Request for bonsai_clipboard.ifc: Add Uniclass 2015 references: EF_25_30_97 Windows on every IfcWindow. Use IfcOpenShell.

First a look at what the model holds.

```python
import ifcopenshell

model = ifcopenshell.open("bonsai_clipboard.ifc")
print(model.schema)
print("classifications:", [c.Name for c in model.by_type("IfcClassification")])
for ifc_class in ("IfcDoor", "IfcRoof", "IfcStair", "IfcWall", "IfcWindow"):
    print(ifc_class, len(model.by_type(ifc_class)))
```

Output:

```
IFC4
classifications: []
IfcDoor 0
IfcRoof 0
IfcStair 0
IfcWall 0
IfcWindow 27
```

```python
import ifcopenshell
import ifcopenshell.api.classification

model = ifcopenshell.open("bonsai_clipboard.ifc")

system = ifcopenshell.api.classification.add_classification(model, classification="Uniclass 2015")

codes = {
    "IfcWindow": ("EF_25_30_97", "Windows"),
}
for ifc_class, (code, name) in codes.items():
    products = model.by_type(ifc_class)
    ifcopenshell.api.classification.add_reference(
        model, products=products, classification=system, identification=code, name=name
    )
    print(code, len(products))

model.write("bonsai_clipboard_v2.ifc")
```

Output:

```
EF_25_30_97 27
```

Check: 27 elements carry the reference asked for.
